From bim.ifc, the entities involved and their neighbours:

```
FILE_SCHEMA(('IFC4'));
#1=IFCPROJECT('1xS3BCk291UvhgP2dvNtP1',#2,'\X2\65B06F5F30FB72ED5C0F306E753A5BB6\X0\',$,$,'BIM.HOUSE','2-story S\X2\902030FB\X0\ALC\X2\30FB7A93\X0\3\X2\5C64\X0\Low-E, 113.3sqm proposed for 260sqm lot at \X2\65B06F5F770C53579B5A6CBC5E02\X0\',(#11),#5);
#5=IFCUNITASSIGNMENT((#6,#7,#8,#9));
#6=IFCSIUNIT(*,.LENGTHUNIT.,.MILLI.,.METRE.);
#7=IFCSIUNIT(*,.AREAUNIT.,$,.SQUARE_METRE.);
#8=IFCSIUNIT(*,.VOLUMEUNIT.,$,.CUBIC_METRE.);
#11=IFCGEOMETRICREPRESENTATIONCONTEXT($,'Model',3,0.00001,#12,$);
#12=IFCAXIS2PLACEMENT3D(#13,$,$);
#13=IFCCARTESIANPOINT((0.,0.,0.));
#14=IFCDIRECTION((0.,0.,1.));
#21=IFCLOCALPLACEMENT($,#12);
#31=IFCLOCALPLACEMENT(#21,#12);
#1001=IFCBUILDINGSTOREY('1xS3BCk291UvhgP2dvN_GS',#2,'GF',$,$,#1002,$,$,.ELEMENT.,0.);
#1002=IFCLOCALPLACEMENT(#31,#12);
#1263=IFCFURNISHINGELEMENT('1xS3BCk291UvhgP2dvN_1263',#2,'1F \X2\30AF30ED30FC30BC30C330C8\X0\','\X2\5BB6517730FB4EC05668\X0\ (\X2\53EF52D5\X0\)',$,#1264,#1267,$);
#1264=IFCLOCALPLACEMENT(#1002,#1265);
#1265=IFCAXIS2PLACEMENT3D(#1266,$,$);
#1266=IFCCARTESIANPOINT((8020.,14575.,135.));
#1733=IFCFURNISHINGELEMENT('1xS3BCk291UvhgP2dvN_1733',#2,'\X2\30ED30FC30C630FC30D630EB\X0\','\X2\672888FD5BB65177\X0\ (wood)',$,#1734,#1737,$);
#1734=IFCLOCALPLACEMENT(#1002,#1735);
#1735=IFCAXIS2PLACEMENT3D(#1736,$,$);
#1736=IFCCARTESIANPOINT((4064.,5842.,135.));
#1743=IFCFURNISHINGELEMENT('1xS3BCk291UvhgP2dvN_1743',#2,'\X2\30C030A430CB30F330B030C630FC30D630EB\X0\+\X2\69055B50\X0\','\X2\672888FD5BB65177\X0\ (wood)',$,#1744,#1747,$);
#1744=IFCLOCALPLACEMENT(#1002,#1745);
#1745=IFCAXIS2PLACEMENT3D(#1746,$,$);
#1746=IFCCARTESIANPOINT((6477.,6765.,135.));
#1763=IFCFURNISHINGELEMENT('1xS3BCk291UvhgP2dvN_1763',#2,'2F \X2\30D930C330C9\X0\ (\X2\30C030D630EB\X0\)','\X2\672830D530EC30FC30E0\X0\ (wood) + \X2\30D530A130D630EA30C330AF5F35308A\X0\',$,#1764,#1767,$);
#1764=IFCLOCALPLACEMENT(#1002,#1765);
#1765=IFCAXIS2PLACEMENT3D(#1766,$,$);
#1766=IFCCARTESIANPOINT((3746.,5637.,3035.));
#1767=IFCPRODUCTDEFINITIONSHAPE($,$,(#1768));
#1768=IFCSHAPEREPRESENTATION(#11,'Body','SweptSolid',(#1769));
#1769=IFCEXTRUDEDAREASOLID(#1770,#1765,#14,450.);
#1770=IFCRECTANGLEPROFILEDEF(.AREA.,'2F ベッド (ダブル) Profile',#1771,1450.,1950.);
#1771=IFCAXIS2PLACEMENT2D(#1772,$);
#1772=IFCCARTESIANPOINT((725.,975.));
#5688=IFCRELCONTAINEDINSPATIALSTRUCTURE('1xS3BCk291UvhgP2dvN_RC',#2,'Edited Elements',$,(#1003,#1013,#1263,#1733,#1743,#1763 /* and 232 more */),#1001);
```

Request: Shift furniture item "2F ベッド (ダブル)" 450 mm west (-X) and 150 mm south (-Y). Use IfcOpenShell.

```python
import ifcopenshell
import ifcopenshell.api.geometry
import ifcopenshell.util.placement
import ifcopenshell.util.unit

model = ifcopenshell.open("bim.ifc")
unit_scale = ifcopenshell.util.unit.calculate_unit_scale(model)

item = model.by_guid("1xS3BCk291UvhgP2dvN_1763")
matrix = ifcopenshell.util.placement.get_local_placement(item.ObjectPlacement)
matrix[0, 3] -= 0.45 / unit_scale
matrix[1, 3] -= 0.15 / unit_scale
ifcopenshell.api.geometry.edit_object_placement(model, product=item, matrix=matrix, is_si=False)

print(ifcopenshell.util.placement.get_local_placement(item.ObjectPlacement).round(3) + 0.0)

model.write("bim_updated.ifc")
```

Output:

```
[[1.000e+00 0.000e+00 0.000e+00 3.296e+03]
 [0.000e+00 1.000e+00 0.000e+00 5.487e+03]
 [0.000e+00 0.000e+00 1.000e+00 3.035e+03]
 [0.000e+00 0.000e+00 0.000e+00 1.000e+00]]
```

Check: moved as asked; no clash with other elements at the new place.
